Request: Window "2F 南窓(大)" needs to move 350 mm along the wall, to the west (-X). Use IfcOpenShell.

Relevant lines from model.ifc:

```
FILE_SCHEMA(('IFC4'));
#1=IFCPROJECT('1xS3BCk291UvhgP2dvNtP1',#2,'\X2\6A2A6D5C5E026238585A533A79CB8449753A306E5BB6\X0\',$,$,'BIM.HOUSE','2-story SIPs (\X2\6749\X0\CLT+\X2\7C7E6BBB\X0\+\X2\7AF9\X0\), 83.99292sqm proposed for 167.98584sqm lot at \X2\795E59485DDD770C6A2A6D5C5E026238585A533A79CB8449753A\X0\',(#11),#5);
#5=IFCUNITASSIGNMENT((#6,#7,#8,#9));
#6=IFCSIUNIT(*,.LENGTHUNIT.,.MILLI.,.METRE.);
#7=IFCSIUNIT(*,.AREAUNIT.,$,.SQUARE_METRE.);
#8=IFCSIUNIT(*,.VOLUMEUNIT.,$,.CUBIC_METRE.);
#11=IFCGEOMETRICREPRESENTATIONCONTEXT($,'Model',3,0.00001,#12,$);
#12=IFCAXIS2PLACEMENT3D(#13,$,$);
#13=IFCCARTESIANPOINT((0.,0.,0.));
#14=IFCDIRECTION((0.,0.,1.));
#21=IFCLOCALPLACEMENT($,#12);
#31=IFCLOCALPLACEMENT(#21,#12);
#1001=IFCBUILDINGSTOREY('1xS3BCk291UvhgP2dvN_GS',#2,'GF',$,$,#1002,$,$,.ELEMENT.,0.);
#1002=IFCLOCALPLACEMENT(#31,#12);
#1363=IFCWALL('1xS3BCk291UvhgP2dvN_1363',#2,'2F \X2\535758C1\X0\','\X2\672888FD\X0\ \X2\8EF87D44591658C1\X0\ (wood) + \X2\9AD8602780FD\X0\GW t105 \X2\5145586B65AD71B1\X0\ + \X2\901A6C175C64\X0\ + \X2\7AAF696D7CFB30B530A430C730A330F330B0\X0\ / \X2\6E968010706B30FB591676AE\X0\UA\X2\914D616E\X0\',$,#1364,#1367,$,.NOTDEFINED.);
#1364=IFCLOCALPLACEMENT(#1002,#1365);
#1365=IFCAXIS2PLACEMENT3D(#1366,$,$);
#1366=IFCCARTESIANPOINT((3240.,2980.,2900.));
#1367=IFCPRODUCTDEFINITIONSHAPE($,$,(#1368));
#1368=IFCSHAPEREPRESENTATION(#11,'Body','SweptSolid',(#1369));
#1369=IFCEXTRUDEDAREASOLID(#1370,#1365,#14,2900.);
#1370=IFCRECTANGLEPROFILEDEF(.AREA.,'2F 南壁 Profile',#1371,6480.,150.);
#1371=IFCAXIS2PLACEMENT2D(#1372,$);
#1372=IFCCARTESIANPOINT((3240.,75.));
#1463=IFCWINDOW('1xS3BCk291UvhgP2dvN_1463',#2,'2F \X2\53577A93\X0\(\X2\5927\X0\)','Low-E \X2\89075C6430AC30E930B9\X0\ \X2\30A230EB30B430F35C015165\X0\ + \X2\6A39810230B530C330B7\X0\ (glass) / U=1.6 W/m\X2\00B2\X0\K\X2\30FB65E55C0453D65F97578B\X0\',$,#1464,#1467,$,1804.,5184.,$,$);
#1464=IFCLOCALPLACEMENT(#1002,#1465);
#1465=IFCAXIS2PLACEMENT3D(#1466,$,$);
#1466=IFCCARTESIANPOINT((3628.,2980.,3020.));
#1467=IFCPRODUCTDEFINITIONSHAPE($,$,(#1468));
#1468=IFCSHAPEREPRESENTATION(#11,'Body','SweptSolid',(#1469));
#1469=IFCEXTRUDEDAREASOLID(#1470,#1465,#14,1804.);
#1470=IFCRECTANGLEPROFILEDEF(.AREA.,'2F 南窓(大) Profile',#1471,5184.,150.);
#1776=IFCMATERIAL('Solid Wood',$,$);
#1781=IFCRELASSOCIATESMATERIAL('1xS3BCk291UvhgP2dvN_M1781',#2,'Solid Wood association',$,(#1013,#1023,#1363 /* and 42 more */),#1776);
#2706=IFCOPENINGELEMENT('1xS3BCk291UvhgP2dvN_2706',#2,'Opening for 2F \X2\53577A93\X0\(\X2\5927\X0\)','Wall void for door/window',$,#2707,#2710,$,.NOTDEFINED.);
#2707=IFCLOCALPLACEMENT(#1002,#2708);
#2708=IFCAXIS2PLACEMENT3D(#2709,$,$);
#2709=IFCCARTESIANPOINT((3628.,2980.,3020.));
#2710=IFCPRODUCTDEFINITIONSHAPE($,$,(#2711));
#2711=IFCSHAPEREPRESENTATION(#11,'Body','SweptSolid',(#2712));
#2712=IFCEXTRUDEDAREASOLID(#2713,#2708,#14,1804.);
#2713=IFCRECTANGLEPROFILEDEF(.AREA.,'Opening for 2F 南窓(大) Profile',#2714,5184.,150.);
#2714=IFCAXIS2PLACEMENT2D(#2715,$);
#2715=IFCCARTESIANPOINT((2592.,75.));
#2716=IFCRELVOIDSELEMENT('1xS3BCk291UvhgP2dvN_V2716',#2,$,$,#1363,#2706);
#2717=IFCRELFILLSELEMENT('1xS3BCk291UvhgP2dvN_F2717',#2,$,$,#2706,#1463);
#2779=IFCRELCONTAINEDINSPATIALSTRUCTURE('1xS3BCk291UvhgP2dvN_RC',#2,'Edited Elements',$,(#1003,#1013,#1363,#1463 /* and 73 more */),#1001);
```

```python
import ifcopenshell
import ifcopenshell.api.geometry
import ifcopenshell.util.placement
import ifcopenshell.util.unit

model = ifcopenshell.open("model.ifc")
unit_scale = ifcopenshell.util.unit.calculate_unit_scale(model)

window = model.by_guid("1xS3BCk291UvhgP2dvN_1463")
opening = window.FillsVoids[0].RelatingOpeningElement
wall = opening.VoidsElements[0].RelatingBuildingElement

wall_matrix = ifcopenshell.util.placement.get_local_placement(wall.ObjectPlacement)
shift = wall_matrix[:3, 0] * -0.35 / unit_scale
before = ifcopenshell.util.placement.get_local_placement(window.ObjectPlacement)[:3, 3].copy()

# The window is not placed relative to its opening, so move both.
for product in (opening, window):
    matrix = ifcopenshell.util.placement.get_local_placement(product.ObjectPlacement)
    matrix[:3, 3] += shift
    ifcopenshell.api.geometry.edit_object_placement(model, product=product, matrix=matrix, is_si=False)

after = ifcopenshell.util.placement.get_local_placement(window.ObjectPlacement)[:3, 3]
print("window moved by", (after - before).round(3) + 0.0)

model.write("model_rev.ifc")
```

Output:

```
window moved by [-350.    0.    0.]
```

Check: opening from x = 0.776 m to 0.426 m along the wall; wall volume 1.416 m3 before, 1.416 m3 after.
